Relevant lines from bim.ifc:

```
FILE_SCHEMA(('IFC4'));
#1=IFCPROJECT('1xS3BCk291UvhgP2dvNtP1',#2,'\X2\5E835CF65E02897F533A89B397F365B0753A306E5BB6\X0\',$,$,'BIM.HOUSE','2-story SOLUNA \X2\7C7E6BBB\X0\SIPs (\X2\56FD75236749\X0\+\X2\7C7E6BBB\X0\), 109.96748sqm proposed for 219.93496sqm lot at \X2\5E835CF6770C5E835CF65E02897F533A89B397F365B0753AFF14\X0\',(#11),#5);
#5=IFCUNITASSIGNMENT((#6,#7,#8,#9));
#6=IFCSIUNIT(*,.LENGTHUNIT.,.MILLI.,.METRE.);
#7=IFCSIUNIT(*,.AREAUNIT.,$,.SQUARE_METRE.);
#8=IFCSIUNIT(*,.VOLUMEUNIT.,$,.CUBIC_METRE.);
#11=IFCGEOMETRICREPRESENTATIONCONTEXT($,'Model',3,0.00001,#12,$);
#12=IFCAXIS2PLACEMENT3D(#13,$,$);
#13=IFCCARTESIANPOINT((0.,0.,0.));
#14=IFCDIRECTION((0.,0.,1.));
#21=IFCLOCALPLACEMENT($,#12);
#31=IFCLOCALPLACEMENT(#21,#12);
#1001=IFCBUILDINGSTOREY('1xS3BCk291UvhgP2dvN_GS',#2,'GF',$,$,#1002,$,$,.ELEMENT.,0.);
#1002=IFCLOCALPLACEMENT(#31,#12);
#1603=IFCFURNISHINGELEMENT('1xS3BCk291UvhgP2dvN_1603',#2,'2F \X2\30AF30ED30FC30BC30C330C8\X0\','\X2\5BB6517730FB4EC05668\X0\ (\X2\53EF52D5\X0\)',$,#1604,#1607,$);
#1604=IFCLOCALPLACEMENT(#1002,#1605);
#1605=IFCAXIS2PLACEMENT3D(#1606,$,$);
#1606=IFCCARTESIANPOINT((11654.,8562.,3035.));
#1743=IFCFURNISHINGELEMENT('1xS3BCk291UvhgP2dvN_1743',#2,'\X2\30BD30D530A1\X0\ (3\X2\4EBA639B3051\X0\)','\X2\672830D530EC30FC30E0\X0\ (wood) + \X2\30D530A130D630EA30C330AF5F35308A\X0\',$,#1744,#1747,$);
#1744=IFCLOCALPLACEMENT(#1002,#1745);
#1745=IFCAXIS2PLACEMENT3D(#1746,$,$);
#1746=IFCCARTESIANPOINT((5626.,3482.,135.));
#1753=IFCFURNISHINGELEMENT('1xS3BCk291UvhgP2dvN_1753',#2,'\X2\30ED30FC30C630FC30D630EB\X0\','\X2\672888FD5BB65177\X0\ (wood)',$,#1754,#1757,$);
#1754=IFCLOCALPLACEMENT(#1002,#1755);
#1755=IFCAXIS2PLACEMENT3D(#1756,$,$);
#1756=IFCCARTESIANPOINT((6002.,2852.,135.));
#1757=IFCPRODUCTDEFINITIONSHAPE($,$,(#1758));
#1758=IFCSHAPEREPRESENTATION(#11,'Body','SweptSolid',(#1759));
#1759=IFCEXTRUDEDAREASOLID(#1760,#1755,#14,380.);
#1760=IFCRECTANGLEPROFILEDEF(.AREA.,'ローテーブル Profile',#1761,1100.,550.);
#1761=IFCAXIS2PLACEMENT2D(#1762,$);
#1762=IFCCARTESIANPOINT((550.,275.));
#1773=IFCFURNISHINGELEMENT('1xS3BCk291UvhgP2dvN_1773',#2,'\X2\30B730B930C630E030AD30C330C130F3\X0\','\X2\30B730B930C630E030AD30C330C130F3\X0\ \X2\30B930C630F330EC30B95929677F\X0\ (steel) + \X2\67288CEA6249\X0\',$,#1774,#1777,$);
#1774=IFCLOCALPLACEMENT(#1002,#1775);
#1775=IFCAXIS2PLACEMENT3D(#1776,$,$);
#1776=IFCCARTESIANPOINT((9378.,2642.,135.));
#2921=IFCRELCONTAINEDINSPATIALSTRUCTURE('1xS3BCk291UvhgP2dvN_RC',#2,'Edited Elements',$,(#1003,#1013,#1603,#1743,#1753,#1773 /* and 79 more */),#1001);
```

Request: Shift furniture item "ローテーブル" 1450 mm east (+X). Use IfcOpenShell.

```python
import ifcopenshell
import ifcopenshell.api.geometry
import ifcopenshell.util.placement
import ifcopenshell.util.unit

model = ifcopenshell.open("bim.ifc")
unit_scale = ifcopenshell.util.unit.calculate_unit_scale(model)

item = model.by_id(1753)
matrix = ifcopenshell.util.placement.get_local_placement(item.ObjectPlacement)
matrix[0, 3] += 1.45 / unit_scale
ifcopenshell.api.geometry.edit_object_placement(model, product=item, matrix=matrix, is_si=False)

print(ifcopenshell.util.placement.get_local_placement(item.ObjectPlacement).round(3) + 0.0)

model.write("bim_updated.ifc")
```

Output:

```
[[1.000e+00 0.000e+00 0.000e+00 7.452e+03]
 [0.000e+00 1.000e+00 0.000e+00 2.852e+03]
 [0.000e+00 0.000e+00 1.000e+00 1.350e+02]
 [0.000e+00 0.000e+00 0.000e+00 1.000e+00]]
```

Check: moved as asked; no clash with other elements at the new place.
